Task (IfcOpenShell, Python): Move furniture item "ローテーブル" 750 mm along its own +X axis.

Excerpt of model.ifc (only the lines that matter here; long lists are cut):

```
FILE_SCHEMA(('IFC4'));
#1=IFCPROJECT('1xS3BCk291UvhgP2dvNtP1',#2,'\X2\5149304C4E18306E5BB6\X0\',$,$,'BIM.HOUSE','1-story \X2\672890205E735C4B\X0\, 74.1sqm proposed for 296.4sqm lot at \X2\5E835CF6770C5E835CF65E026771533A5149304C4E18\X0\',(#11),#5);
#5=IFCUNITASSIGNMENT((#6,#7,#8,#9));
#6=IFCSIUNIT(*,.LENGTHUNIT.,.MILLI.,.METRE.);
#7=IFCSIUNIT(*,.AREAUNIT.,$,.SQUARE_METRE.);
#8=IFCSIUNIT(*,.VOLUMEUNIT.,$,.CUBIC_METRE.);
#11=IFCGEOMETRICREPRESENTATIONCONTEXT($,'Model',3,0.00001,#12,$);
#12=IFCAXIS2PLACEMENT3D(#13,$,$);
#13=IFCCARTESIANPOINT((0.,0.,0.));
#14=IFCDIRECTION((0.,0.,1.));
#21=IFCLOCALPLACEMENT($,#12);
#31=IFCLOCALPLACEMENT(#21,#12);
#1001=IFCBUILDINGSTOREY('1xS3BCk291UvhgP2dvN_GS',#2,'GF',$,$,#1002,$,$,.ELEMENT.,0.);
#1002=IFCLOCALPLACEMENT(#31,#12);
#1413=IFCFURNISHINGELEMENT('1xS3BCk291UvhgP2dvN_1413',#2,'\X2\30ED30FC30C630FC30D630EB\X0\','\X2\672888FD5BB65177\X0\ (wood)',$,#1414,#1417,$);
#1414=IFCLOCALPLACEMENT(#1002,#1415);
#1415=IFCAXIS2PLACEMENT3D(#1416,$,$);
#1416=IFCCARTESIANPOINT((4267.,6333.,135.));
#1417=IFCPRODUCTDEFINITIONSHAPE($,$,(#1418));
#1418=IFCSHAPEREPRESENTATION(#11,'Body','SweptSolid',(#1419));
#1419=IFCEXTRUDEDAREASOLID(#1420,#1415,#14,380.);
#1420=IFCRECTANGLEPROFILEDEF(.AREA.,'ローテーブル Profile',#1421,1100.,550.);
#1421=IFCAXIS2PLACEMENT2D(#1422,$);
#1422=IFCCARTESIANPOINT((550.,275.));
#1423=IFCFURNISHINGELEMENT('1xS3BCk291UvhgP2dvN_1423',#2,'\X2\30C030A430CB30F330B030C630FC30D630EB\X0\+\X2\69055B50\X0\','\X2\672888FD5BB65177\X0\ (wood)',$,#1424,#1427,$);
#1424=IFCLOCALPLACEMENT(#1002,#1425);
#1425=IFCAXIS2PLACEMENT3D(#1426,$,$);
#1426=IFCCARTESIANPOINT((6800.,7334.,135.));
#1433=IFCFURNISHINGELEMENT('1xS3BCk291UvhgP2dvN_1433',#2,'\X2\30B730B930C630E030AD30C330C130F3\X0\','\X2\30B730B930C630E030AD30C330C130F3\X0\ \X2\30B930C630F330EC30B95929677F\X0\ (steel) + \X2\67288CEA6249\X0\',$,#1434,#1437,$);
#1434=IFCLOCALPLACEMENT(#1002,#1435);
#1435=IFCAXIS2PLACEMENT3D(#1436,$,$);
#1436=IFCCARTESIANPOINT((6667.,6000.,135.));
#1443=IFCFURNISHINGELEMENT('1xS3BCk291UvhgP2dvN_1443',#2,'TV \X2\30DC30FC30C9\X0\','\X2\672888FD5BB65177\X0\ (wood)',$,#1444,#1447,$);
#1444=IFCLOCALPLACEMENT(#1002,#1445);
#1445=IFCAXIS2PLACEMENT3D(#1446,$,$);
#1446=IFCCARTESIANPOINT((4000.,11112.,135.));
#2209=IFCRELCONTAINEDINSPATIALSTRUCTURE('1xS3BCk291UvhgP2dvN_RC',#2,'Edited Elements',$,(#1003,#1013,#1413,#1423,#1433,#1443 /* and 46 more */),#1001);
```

```python
import ifcopenshell
import ifcopenshell.api.geometry
import ifcopenshell.util.placement
import ifcopenshell.util.unit

model = ifcopenshell.open("model.ifc")
unit_scale = ifcopenshell.util.unit.calculate_unit_scale(model)

item = model.by_guid("1xS3BCk291UvhgP2dvN_1413")
matrix = ifcopenshell.util.placement.get_local_placement(item.ObjectPlacement)
matrix[:3, 3] += matrix[:3, 0] * 0.75 / unit_scale
ifcopenshell.api.geometry.edit_object_placement(model, product=item, matrix=matrix, is_si=False)

print(ifcopenshell.util.placement.get_local_placement(item.ObjectPlacement).round(3) + 0.0)

model.write("model_rev.ifc")
```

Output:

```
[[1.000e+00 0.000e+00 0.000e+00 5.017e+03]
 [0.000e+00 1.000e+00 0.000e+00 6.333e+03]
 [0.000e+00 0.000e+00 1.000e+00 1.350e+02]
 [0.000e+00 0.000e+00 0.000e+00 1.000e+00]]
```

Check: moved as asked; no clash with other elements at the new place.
